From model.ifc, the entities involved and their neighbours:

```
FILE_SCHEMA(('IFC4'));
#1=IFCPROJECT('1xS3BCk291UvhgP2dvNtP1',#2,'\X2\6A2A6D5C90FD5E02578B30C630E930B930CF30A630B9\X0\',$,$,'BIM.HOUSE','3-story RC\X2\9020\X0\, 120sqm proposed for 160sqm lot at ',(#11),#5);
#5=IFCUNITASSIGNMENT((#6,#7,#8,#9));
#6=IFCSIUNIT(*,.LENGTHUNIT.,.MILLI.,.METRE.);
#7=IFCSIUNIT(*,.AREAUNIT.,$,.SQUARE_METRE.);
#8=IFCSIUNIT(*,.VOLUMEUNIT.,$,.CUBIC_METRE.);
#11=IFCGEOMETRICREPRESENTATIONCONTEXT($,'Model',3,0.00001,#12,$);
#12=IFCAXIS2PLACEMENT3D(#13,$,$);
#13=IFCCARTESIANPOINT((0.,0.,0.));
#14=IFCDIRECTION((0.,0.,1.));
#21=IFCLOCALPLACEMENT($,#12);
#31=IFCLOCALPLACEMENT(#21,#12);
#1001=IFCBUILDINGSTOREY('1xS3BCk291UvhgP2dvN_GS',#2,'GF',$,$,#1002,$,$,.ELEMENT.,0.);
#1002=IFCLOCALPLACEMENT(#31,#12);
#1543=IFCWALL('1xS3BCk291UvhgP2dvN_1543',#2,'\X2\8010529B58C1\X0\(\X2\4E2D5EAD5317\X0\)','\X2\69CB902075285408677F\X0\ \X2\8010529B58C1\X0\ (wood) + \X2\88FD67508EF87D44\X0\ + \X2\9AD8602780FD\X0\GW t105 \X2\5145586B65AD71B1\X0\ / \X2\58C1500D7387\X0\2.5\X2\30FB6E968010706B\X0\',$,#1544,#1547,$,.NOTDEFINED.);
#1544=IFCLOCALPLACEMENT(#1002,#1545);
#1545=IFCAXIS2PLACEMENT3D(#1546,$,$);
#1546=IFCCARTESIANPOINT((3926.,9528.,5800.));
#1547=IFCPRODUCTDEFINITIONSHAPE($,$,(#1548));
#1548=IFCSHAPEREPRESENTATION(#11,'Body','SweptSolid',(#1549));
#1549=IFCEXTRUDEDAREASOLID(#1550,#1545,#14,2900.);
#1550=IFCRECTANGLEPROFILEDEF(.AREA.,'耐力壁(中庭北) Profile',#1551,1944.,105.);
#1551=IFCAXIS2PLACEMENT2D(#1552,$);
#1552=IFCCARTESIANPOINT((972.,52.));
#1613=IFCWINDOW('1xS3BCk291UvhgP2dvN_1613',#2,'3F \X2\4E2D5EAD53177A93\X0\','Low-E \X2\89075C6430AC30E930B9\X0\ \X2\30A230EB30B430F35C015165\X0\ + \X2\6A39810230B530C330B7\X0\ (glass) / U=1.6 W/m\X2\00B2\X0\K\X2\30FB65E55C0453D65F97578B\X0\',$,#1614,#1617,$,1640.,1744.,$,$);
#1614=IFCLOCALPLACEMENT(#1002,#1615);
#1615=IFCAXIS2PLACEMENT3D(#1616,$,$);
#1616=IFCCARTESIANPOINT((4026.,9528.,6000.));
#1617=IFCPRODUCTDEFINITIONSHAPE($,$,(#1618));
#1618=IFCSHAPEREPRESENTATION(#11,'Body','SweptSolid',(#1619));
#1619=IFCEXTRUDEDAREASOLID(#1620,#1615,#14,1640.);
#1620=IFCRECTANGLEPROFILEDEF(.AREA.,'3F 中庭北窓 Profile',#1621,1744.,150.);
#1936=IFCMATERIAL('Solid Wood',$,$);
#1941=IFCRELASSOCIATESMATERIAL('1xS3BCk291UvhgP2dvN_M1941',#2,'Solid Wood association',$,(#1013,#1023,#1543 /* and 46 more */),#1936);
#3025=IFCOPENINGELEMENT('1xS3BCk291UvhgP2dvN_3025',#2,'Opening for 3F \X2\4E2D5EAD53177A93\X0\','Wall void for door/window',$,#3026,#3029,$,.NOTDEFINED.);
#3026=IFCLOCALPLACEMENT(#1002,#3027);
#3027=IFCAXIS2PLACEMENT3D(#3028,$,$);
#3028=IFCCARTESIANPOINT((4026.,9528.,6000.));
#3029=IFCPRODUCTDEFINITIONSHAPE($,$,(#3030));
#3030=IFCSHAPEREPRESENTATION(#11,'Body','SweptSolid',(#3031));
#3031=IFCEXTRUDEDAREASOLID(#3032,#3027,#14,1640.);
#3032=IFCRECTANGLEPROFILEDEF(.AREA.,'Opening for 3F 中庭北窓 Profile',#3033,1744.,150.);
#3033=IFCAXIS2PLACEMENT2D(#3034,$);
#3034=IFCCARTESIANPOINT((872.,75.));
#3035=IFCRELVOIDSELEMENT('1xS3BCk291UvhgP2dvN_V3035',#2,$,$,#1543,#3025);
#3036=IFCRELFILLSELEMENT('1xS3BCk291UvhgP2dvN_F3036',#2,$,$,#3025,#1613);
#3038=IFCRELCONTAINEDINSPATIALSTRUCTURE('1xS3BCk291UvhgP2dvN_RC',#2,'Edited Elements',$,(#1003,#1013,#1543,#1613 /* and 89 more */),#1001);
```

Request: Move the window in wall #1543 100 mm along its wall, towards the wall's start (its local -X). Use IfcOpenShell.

```python
import ifcopenshell
import ifcopenshell.api.geometry
import ifcopenshell.util.placement
import ifcopenshell.util.unit

model = ifcopenshell.open("model.ifc")
unit_scale = ifcopenshell.util.unit.calculate_unit_scale(model)

window = model.by_id(1613)
opening = window.FillsVoids[0].RelatingOpeningElement
wall = opening.VoidsElements[0].RelatingBuildingElement

wall_matrix = ifcopenshell.util.placement.get_local_placement(wall.ObjectPlacement)
shift = wall_matrix[:3, 0] * -0.1 / unit_scale
before = ifcopenshell.util.placement.get_local_placement(window.ObjectPlacement)[:3, 3].copy()

# The window is not placed relative to its opening, so move both.
for product in (opening, window):
    matrix = ifcopenshell.util.placement.get_local_placement(product.ObjectPlacement)
    matrix[:3, 3] += shift
    ifcopenshell.api.geometry.edit_object_placement(model, product=product, matrix=matrix, is_si=False)

after = ifcopenshell.util.placement.get_local_placement(window.ObjectPlacement)[:3, 3]
print("window moved by", (after - before).round(3) + 0.0)

model.write("model-out.ifc")
```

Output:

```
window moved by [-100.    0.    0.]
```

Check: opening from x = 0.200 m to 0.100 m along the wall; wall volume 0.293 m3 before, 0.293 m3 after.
